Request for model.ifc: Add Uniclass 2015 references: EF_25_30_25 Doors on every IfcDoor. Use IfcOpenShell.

First a look at what the model holds.

```python
import ifcopenshell

model = ifcopenshell.open("model.ifc")
print(model.schema)
print("classifications:", [c.Name for c in model.by_type("IfcClassification")])
for ifc_class in ("IfcDoor", "IfcRoof", "IfcStair", "IfcWall", "IfcWindow"):
    print(ifc_class, len(model.by_type(ifc_class)))
```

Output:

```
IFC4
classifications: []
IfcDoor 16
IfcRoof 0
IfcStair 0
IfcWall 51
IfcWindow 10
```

```python
import ifcopenshell
import ifcopenshell.api.classification

model = ifcopenshell.open("model.ifc")

system = ifcopenshell.api.classification.add_classification(model, classification="Uniclass 2015")

codes = {
    "IfcDoor": ("EF_25_30_25", "Doors"),
}
for ifc_class, (code, name) in codes.items():
    products = model.by_type(ifc_class)
    ifcopenshell.api.classification.add_reference(
        model, products=products, classification=system, identification=code, name=name
    )
    print(code, len(products))

model.write("model_v2.ifc")
```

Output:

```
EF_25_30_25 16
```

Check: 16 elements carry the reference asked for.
